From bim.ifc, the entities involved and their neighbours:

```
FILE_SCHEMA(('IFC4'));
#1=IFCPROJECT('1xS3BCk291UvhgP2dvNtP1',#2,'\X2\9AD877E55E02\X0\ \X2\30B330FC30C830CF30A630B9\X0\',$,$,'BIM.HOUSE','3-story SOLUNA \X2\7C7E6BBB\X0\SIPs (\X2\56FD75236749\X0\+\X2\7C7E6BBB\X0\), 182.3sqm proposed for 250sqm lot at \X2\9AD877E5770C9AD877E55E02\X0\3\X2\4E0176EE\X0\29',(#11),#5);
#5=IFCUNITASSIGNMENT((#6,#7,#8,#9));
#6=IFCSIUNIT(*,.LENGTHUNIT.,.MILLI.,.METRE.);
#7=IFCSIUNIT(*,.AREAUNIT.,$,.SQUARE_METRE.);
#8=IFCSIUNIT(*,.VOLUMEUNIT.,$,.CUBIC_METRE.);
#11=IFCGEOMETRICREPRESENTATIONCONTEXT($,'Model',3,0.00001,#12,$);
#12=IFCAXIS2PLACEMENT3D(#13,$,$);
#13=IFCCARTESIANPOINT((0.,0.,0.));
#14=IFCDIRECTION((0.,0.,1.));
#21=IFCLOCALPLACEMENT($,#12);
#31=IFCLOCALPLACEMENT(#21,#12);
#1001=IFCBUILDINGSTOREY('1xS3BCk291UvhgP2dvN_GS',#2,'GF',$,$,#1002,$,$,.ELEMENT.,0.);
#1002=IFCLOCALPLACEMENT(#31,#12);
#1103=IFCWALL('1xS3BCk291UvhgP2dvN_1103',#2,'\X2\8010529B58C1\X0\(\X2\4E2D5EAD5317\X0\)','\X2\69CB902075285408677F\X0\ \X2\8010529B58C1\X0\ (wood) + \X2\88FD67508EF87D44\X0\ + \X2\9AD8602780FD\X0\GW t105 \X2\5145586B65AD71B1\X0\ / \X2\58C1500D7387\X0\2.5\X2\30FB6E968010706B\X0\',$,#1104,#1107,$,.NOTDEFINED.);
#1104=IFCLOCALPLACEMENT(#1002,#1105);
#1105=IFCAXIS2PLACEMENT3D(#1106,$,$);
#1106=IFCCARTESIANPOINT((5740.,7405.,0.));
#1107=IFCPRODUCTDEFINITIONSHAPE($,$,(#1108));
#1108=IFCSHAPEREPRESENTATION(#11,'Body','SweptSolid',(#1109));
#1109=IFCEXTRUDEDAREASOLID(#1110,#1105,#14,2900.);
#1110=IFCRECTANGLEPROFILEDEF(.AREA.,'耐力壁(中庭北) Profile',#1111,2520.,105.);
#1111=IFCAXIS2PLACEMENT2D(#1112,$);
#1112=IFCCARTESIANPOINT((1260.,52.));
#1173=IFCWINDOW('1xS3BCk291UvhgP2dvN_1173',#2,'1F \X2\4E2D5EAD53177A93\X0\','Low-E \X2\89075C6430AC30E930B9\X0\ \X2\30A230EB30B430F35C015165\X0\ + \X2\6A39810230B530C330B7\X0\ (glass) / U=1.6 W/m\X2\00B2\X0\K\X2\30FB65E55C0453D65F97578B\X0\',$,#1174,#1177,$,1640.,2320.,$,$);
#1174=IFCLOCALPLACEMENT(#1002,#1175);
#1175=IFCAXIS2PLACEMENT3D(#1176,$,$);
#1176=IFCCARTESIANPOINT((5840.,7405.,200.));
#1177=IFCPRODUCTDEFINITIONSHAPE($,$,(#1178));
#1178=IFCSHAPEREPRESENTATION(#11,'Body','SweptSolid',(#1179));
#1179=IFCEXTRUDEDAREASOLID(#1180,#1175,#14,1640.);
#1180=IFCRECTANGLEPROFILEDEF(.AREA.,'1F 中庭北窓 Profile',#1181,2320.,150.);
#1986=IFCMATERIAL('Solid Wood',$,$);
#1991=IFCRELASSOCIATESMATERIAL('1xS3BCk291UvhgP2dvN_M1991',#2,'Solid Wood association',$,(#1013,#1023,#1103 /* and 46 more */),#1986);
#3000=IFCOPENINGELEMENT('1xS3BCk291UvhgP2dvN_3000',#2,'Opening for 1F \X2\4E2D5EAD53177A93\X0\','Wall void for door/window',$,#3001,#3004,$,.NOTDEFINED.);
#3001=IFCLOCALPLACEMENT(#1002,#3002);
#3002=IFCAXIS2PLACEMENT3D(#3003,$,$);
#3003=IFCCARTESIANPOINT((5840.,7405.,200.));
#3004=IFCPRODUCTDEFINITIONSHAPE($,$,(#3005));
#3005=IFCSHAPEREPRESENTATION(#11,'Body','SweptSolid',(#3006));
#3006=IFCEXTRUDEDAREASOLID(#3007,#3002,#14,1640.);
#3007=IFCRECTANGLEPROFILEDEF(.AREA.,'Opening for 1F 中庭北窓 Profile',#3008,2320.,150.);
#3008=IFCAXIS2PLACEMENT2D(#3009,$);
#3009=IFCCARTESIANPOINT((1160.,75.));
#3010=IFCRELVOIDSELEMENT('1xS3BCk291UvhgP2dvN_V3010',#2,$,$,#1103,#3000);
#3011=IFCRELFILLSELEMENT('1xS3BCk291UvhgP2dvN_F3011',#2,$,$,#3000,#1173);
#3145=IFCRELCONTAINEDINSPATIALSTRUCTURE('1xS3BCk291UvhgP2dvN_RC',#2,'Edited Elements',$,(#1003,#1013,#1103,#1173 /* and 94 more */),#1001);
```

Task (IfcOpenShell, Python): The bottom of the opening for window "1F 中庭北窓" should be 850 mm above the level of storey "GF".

```python
import numpy as np
import ifcopenshell
import ifcopenshell.api.geometry
import ifcopenshell.geom
import ifcopenshell.util.element
import ifcopenshell.util.placement
import ifcopenshell.util.shape
import ifcopenshell.util.unit

model = ifcopenshell.open("bim.ifc")
unit_scale = ifcopenshell.util.unit.calculate_unit_scale(model)

window = model.by_guid("1xS3BCk291UvhgP2dvN_1173")
opening = window.FillsVoids[0].RelatingOpeningElement
storey = ifcopenshell.util.element.get_container(window, ifc_class="IfcBuildingStorey")
level = ifcopenshell.util.placement.get_local_placement(storey.ObjectPlacement)[2, 3]

# The opening's origin need not be at the sill, so measure its lowest point.
shape = ifcopenshell.geom.create_shape(ifcopenshell.geom.settings(), opening)
bottom = ifcopenshell.util.shape.get_shape_bottom_elevation(shape, shape.geometry) / unit_scale
dz = level + 850.0 - bottom

shift = np.array([0.0, 0.0, dz])
# The window is not placed relative to its opening, so move both.
for product in (opening, window):
    matrix = ifcopenshell.util.placement.get_local_placement(product.ObjectPlacement)
    matrix[:3, 3] += shift
    ifcopenshell.api.geometry.edit_object_placement(model, product=product, matrix=matrix, is_si=False)

print(f"moved by {dz * unit_scale:+.3f} m")

model.write("bim_v2.ifc")
```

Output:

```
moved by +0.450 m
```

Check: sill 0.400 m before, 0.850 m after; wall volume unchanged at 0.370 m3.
